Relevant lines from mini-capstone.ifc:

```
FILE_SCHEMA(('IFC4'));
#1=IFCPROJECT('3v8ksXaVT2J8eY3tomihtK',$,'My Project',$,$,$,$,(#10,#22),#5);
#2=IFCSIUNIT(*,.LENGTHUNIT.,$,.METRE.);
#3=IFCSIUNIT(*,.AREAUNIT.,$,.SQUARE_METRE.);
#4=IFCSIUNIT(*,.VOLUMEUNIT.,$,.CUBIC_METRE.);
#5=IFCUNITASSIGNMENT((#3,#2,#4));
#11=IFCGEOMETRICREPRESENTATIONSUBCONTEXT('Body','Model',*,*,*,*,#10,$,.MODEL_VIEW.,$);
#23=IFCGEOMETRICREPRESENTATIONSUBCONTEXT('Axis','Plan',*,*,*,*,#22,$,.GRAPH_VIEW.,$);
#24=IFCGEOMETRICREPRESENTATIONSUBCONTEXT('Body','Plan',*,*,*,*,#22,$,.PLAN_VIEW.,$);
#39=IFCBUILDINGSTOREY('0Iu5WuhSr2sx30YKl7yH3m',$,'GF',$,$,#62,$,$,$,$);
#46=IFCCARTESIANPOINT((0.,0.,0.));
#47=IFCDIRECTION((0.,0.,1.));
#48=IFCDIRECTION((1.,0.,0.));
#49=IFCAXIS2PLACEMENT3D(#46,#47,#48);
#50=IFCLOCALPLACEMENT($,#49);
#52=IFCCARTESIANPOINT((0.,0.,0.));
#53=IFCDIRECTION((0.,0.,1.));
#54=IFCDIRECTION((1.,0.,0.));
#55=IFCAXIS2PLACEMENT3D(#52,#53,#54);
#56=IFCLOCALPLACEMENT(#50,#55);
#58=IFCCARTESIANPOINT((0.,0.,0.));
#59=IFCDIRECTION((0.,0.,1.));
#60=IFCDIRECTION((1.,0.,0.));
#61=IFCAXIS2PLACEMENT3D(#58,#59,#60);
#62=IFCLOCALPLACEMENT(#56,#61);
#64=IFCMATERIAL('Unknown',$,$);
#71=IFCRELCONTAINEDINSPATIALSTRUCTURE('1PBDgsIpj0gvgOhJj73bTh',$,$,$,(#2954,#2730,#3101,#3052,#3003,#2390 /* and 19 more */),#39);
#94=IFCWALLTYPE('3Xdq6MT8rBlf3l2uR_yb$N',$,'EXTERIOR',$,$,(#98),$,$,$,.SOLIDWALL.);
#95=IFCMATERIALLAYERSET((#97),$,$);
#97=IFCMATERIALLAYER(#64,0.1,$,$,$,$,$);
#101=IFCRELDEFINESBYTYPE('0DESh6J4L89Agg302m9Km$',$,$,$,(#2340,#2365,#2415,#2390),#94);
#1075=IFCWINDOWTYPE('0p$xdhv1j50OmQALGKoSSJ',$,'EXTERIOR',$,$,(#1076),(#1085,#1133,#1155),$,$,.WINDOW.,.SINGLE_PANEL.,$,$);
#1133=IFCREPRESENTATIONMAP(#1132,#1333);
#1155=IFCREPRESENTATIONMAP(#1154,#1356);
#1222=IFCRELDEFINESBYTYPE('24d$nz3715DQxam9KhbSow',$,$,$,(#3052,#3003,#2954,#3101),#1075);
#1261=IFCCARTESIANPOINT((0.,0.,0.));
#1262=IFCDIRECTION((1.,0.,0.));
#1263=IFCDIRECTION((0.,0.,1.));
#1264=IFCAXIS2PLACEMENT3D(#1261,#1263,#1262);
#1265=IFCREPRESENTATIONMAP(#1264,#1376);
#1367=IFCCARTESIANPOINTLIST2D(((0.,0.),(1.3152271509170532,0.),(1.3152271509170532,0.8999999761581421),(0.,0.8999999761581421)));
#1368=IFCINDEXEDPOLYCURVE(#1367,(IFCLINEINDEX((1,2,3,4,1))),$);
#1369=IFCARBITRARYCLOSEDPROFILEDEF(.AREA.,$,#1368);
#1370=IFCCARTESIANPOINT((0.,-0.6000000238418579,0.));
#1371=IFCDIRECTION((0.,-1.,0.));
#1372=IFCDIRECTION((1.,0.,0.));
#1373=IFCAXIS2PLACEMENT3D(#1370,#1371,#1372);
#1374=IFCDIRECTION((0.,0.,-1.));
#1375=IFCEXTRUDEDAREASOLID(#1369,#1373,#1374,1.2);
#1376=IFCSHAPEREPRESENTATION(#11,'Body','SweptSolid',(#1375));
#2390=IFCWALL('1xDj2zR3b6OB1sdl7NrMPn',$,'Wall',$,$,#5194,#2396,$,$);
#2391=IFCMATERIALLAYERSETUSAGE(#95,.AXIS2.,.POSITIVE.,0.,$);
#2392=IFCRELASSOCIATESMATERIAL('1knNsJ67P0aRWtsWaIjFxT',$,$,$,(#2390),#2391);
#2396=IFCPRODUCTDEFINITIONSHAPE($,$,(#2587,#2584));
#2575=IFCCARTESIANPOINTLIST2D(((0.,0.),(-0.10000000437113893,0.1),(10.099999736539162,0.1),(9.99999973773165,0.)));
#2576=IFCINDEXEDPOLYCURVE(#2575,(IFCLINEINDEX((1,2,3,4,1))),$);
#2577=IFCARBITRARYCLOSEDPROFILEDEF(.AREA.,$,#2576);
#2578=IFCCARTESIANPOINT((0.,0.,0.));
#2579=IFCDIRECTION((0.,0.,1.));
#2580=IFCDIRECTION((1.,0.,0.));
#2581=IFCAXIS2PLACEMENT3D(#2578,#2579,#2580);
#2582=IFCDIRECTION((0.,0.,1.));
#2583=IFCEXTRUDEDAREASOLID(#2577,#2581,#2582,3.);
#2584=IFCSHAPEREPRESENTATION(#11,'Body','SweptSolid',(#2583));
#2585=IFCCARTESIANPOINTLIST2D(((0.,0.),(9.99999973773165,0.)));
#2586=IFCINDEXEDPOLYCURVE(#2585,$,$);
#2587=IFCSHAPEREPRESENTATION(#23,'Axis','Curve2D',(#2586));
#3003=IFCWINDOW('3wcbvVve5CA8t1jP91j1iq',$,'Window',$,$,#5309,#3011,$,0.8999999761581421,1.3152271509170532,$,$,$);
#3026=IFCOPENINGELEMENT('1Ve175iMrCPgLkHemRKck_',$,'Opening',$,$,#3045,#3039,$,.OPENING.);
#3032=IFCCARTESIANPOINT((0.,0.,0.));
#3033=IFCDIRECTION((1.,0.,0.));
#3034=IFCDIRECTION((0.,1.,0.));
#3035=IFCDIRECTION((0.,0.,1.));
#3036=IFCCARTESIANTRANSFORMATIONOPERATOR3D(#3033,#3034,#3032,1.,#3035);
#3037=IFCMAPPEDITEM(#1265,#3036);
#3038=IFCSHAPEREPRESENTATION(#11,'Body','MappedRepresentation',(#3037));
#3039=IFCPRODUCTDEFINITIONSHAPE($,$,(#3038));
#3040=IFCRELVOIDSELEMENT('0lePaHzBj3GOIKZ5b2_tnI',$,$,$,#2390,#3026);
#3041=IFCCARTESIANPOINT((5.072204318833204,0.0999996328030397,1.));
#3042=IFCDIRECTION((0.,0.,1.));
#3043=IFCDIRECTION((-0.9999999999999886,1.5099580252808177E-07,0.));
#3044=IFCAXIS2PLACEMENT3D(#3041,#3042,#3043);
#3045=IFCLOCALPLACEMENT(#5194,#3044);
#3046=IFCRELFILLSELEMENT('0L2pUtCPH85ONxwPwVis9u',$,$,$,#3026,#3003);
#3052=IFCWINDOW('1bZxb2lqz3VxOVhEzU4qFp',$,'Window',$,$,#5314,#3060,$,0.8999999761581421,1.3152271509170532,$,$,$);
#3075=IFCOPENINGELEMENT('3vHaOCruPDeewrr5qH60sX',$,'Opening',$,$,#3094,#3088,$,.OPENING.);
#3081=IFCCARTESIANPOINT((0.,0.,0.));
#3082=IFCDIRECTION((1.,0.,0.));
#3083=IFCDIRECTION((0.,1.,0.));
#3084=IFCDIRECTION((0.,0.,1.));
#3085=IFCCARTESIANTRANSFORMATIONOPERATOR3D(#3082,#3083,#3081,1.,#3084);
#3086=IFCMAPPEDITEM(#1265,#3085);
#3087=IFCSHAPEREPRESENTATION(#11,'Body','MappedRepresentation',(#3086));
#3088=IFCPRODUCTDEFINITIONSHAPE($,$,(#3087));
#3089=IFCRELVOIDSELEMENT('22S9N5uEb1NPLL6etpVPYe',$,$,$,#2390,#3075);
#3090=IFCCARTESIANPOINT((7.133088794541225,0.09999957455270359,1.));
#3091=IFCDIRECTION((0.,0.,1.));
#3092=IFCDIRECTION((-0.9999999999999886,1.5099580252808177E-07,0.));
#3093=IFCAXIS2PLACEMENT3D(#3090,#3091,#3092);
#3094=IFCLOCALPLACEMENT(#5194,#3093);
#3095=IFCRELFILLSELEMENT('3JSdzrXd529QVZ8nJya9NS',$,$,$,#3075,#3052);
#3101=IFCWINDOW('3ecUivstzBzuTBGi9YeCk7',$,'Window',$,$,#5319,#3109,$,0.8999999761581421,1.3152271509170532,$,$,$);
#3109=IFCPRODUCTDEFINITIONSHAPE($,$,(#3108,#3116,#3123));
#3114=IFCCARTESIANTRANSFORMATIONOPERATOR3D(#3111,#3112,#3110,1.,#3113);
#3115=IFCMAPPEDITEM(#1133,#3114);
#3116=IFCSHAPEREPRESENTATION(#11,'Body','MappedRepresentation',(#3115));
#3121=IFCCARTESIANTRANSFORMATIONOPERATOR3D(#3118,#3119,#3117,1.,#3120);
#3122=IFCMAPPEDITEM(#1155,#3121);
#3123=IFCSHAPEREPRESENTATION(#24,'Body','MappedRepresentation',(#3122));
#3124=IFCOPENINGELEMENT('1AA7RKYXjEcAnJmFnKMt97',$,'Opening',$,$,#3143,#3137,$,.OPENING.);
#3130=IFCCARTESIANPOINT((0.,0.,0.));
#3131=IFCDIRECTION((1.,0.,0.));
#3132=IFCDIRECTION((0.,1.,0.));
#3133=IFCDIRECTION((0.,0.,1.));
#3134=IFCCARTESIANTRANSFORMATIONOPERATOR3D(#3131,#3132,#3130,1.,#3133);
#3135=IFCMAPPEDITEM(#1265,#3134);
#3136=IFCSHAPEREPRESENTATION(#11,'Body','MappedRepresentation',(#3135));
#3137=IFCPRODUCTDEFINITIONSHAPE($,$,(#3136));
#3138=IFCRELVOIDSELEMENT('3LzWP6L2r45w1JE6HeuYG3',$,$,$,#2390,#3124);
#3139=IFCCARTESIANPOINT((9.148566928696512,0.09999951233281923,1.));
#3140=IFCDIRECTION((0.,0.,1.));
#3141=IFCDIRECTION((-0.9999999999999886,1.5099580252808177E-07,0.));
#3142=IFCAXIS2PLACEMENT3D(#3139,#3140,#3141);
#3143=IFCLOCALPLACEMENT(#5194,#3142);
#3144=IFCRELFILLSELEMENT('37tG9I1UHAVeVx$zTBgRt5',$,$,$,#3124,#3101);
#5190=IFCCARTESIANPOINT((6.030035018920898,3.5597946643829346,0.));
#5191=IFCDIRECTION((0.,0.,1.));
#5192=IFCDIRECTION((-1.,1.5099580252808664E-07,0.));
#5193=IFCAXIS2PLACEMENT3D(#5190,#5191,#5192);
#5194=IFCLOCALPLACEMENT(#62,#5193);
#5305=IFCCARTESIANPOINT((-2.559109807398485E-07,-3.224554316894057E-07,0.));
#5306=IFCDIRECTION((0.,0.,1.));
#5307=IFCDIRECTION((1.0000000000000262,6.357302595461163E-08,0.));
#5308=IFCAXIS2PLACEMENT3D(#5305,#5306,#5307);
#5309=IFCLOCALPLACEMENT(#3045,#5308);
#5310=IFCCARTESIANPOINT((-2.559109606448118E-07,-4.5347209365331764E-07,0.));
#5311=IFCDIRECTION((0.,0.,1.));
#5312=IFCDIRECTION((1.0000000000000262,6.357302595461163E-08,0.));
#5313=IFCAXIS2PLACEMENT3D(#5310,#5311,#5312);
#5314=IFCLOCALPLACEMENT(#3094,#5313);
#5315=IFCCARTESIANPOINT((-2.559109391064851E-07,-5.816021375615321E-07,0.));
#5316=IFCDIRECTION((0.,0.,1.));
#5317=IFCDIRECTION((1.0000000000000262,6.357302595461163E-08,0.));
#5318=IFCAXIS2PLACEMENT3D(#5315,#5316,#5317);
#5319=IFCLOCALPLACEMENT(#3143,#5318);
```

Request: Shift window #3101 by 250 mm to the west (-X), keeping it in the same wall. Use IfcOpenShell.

```python
import ifcopenshell
import ifcopenshell.api.geometry
import ifcopenshell.util.placement
import ifcopenshell.util.unit

model = ifcopenshell.open("mini-capstone.ifc")
unit_scale = ifcopenshell.util.unit.calculate_unit_scale(model)

window = model.by_guid("3ecUivstzBzuTBGi9YeCk7")
opening = window.FillsVoids[0].RelatingOpeningElement
wall = opening.VoidsElements[0].RelatingBuildingElement

wall_matrix = ifcopenshell.util.placement.get_local_placement(wall.ObjectPlacement)
shift = wall_matrix[:3, 0] * 0.25 / unit_scale
before = ifcopenshell.util.placement.get_local_placement(window.ObjectPlacement)[:3, 3].copy()

# The window is placed relative to its opening, so it follows when the opening moves.
matrix = ifcopenshell.util.placement.get_local_placement(opening.ObjectPlacement)
matrix[:3, 3] += shift
ifcopenshell.api.geometry.edit_object_placement(
    model, product=opening, matrix=matrix, is_si=False, should_transform_children=True
)

after = ifcopenshell.util.placement.get_local_placement(window.ObjectPlacement)[:3, 3]
print("window moved by", (after - before).round(3) + 0.0)

model.write("mini-capstone-out.ifc")
```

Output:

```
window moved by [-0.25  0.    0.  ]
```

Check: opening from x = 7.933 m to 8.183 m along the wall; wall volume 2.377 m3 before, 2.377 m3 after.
